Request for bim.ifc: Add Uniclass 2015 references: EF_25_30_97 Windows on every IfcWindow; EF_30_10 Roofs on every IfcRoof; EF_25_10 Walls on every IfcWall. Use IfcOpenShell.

First a look at what the model holds.

```python
import ifcopenshell

model = ifcopenshell.open("bim.ifc")
print(model.schema)
print("classifications:", [c.Name for c in model.by_type("IfcClassification")])
for ifc_class in ("IfcDoor", "IfcRoof", "IfcStair", "IfcWall", "IfcWindow"):
    print(ifc_class, len(model.by_type(ifc_class)))
```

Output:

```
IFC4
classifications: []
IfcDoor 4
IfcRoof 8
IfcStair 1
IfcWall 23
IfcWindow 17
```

```python
import ifcopenshell
import ifcopenshell.api.classification

model = ifcopenshell.open("bim.ifc")

system = ifcopenshell.api.classification.add_classification(model, classification="Uniclass 2015")

codes = {
    "IfcWindow": ("EF_25_30_97", "Windows"),
    "IfcRoof": ("EF_30_10", "Roofs"),
    "IfcWall": ("EF_25_10", "Walls"),
}
for ifc_class, (code, name) in codes.items():
    products = model.by_type(ifc_class)
    ifcopenshell.api.classification.add_reference(
        model, products=products, classification=system, identification=code, name=name
    )
    print(code, len(products))

model.write("bim_rev.ifc")
```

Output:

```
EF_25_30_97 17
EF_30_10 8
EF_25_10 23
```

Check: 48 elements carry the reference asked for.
